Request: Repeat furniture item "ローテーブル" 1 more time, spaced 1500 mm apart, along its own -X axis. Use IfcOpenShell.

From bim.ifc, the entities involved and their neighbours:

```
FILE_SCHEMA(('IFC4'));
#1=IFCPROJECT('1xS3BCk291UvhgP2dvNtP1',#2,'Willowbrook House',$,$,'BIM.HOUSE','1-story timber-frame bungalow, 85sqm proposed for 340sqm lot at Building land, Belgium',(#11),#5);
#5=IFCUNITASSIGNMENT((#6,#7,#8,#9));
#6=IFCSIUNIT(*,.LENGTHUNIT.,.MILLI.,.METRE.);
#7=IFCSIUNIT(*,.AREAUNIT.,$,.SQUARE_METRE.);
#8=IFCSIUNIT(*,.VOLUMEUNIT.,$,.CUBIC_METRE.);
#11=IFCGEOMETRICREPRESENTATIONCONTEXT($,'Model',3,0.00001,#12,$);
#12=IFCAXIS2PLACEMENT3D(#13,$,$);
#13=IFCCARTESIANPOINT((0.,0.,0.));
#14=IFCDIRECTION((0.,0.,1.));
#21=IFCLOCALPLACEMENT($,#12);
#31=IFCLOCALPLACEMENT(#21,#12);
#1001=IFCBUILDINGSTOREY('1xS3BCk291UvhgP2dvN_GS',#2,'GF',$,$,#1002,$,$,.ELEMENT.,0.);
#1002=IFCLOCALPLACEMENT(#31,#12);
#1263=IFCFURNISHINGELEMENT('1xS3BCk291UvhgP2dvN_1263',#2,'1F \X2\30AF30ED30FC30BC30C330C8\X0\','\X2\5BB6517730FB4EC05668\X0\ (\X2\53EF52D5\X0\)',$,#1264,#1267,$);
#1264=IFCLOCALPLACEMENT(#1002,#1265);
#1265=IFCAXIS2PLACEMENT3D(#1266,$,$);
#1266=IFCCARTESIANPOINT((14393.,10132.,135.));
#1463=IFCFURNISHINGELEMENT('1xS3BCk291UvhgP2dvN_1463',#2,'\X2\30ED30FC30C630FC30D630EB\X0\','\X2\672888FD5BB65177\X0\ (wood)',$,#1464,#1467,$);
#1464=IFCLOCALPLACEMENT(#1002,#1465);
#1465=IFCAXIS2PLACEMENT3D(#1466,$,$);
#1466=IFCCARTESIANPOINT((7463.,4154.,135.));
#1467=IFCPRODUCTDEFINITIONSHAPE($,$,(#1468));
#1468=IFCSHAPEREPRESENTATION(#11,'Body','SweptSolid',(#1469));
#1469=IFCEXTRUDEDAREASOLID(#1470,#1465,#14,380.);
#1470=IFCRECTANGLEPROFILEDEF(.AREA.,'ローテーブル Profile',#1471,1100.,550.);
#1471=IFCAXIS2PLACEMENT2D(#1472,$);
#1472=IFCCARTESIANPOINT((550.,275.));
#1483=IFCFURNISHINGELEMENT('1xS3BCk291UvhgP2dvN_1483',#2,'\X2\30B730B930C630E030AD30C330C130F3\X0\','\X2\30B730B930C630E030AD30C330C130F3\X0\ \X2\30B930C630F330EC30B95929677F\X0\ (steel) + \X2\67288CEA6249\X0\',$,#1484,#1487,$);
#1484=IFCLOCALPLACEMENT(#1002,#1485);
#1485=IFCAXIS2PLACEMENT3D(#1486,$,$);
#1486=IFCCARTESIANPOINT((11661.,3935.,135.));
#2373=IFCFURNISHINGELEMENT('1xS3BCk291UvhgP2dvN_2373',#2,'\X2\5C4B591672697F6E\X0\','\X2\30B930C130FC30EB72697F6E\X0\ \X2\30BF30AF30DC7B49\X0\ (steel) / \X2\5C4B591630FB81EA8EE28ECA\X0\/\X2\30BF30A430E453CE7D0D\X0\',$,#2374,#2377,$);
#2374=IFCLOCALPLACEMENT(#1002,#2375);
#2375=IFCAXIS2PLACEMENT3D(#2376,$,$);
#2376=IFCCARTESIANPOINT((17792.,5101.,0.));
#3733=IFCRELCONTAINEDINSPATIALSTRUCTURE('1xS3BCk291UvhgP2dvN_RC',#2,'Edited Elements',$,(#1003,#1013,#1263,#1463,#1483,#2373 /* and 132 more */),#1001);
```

```python
import ifcopenshell
import ifcopenshell.api.geometry
import ifcopenshell.api.root
import ifcopenshell.util.element
import ifcopenshell.util.placement
import ifcopenshell.util.unit

model = ifcopenshell.open("bim.ifc")
unit_scale = ifcopenshell.util.unit.calculate_unit_scale(model)


def reuse_history(source, copy):
    """copy_class also copies each property set's owner history, people and application; keep the originals."""
    for rel in copy.IsDefinedBy:
        if rel.is_a("IfcRelDefinesByProperties") and (history := rel.RelatingPropertyDefinition.OwnerHistory):
            rel.RelatingPropertyDefinition.OwnerHistory = source.OwnerHistory
            ifcopenshell.util.element.remove_deep2(model, history)


source = model.by_guid("1xS3BCk291UvhgP2dvN_1463")
base = ifcopenshell.util.placement.get_local_placement(source.ObjectPlacement)
step = -base[:3, 0] * 1.5 / unit_scale

for i in range(1, 2):
    copy = ifcopenshell.api.root.copy_class(model, product=source)
    copy.Representation = ifcopenshell.util.element.copy_deep(
        model, source.Representation, exclude=["IfcGeometricRepresentationContext", "IfcRepresentationMap"]
    )
    reuse_history(source, copy)
    matrix = base.copy()
    matrix[:3, 3] += i * step
    print("added at", matrix[:3, 3].round(3) + 0.0)
    ifcopenshell.api.geometry.edit_object_placement(model, product=copy, matrix=matrix, is_si=False)

model.write("bim_v2.ifc")
```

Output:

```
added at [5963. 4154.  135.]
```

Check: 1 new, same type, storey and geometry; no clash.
